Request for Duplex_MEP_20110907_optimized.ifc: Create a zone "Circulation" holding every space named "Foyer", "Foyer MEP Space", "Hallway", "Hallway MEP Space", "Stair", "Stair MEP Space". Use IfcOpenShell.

First a look at what the model holds.

```python
import ifcopenshell

model = ifcopenshell.open("Duplex_MEP_20110907_optimized.ifc")
print(model.schema)
seen = {}
for space in model.by_type("IfcSpace"):
    seen[space.LongName] = seen.get(space.LongName, 0) + 1
for name, count in sorted(seen.items(), key=str):
    print(count, "x", name)
print("zones:", [z.Name for z in model.by_type("IfcZone")][:20])
```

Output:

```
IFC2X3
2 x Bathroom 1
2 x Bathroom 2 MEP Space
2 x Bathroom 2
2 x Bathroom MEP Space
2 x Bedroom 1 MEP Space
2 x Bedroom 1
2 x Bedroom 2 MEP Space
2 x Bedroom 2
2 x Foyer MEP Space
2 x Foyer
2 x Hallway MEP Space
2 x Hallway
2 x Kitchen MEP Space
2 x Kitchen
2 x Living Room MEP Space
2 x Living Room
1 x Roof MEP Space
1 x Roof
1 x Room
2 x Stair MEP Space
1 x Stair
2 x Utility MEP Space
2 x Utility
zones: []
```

```python
import ifcopenshell
import ifcopenshell.api.group
import ifcopenshell.api.root

model = ifcopenshell.open("Duplex_MEP_20110907_optimized.ifc")

names = {"Foyer", "Foyer MEP Space", "Hallway", "Hallway MEP Space", "Stair", "Stair MEP Space"}
spaces = [s for s in model.by_type("IfcSpace") if s.LongName in names]

zone = ifcopenshell.api.root.create_entity(model, ifc_class="IfcZone", name="Circulation")
ifcopenshell.api.group.assign_group(model, products=spaces, group=zone)
print(len(spaces), "spaces in", zone.Name)

model.write("Duplex_MEP_20110907_optimized_updated.ifc")
```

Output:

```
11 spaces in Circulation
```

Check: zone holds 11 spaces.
